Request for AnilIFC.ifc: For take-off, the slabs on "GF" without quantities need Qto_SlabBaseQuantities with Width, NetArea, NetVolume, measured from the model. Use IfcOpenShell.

First a look at what the model holds.

```python
import ifcopenshell
import ifcopenshell.util.element
import ifcopenshell.util.unit

model = ifcopenshell.open("AnilIFC.ifc")
print(model.schema)
for unit_type in ("LENGTHUNIT", "AREAUNIT", "VOLUMEUNIT"):
    print(unit_type, ifcopenshell.util.unit.calculate_unit_scale(model, unit_type))
storey = next(s for s in model.by_type("IfcBuildingStorey") if s.Name == "GF")
slabs = [e for e in ifcopenshell.util.element.get_decomposition(storey) if e.is_a("IfcSlab")]
for e in sorted(slabs, key=lambda e: e.id()):
    print(e.id(), e.is_a(), e.Name, list(ifcopenshell.util.element.get_psets(e, qtos_only=True)), sep=" | ")
```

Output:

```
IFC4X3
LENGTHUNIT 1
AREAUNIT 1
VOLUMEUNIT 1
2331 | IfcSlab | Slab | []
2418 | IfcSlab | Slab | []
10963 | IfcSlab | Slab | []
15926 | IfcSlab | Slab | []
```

```python
import ifcopenshell
import ifcopenshell.api.pset
import ifcopenshell.geom
import ifcopenshell.util.element
import ifcopenshell.util.shape
import ifcopenshell.util.unit

model = ifcopenshell.open("AnilIFC.ifc")
unit_scale = ifcopenshell.util.unit.calculate_unit_scale(model)
area_scale = ifcopenshell.util.unit.calculate_unit_scale(model, "AREAUNIT")
volume_scale = ifcopenshell.util.unit.calculate_unit_scale(model, "VOLUMEUNIT")
settings = ifcopenshell.geom.settings()

storey = next(s for s in model.by_type("IfcBuildingStorey") if s.Name == "GF")
slabs = [e for e in ifcopenshell.util.element.get_decomposition(storey) if e.is_a("IfcSlab")]

for e in sorted(slabs, key=lambda e: e.id()):
    if ifcopenshell.util.element.get_psets(e, qtos_only=True, should_inherit=False):
        continue
    # Geometry comes back in metres, in the element's own axes.
    shape = ifcopenshell.geom.create_shape(settings, e)
    values = {
        "Width": ifcopenshell.util.shape.get_z(shape.geometry) / unit_scale,
        "NetArea": ifcopenshell.util.shape.get_footprint_area(shape.geometry) / area_scale,
        "NetVolume": ifcopenshell.util.shape.get_volume(shape.geometry) / volume_scale,
    }
    qto = ifcopenshell.api.pset.add_qto(model, product=e, name="Qto_SlabBaseQuantities")
    ifcopenshell.api.pset.edit_qto(model, qto=qto, properties=values)
    print(e.id(), {k: round(v, 3) for k, v in values.items()})

model.write("AnilIFC_rev.ifc")
```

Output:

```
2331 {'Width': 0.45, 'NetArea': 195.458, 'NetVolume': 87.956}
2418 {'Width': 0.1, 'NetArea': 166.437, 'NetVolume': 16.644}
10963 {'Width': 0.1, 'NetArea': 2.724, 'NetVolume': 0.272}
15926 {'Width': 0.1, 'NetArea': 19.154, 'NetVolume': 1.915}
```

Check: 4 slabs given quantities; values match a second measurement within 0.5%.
